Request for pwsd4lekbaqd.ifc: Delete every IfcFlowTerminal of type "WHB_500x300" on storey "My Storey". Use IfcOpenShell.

First a look at what the model holds.

```python
import ifcopenshell
import ifcopenshell.util.element

model = ifcopenshell.open("pwsd4lekbaqd.ifc")
print(model.schema)
storey = next(s for s in model.by_type("IfcBuildingStorey") if s.Name == "My Storey")
terminals = [e for e in ifcopenshell.util.element.get_decomposition(storey) if e.is_a("IfcFlowTerminal")]
seen = {}
for e in terminals:
    element_type = ifcopenshell.util.element.get_type(e)
    name = element_type.Name if element_type not in (None, e) else None
    seen[name] = seen.get(name, 0) + 1
for name, count in sorted(seen.items(), key=str):
    print(count, "x", name)
```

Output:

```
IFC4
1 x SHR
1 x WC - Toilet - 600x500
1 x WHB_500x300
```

```python
import ifcopenshell
import ifcopenshell.api.root
import ifcopenshell.util.element

model = ifcopenshell.open("pwsd4lekbaqd.ifc")

storey = next(s for s in model.by_type("IfcBuildingStorey") if s.Name == "My Storey")
terminals = [e for e in ifcopenshell.util.element.get_decomposition(storey) if e.is_a("IfcFlowTerminal")]
targets = [e for e in terminals if (t := ifcopenshell.util.element.get_type(e)) not in (None, e) and t.Name == "WHB_500x300"]

for e in targets:
    ifcopenshell.api.root.remove_product(model, product=e)
print(len(targets), "removed")

model.write("pwsd4lekbaqd_edited.ifc")
```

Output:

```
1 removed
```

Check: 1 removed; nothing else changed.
